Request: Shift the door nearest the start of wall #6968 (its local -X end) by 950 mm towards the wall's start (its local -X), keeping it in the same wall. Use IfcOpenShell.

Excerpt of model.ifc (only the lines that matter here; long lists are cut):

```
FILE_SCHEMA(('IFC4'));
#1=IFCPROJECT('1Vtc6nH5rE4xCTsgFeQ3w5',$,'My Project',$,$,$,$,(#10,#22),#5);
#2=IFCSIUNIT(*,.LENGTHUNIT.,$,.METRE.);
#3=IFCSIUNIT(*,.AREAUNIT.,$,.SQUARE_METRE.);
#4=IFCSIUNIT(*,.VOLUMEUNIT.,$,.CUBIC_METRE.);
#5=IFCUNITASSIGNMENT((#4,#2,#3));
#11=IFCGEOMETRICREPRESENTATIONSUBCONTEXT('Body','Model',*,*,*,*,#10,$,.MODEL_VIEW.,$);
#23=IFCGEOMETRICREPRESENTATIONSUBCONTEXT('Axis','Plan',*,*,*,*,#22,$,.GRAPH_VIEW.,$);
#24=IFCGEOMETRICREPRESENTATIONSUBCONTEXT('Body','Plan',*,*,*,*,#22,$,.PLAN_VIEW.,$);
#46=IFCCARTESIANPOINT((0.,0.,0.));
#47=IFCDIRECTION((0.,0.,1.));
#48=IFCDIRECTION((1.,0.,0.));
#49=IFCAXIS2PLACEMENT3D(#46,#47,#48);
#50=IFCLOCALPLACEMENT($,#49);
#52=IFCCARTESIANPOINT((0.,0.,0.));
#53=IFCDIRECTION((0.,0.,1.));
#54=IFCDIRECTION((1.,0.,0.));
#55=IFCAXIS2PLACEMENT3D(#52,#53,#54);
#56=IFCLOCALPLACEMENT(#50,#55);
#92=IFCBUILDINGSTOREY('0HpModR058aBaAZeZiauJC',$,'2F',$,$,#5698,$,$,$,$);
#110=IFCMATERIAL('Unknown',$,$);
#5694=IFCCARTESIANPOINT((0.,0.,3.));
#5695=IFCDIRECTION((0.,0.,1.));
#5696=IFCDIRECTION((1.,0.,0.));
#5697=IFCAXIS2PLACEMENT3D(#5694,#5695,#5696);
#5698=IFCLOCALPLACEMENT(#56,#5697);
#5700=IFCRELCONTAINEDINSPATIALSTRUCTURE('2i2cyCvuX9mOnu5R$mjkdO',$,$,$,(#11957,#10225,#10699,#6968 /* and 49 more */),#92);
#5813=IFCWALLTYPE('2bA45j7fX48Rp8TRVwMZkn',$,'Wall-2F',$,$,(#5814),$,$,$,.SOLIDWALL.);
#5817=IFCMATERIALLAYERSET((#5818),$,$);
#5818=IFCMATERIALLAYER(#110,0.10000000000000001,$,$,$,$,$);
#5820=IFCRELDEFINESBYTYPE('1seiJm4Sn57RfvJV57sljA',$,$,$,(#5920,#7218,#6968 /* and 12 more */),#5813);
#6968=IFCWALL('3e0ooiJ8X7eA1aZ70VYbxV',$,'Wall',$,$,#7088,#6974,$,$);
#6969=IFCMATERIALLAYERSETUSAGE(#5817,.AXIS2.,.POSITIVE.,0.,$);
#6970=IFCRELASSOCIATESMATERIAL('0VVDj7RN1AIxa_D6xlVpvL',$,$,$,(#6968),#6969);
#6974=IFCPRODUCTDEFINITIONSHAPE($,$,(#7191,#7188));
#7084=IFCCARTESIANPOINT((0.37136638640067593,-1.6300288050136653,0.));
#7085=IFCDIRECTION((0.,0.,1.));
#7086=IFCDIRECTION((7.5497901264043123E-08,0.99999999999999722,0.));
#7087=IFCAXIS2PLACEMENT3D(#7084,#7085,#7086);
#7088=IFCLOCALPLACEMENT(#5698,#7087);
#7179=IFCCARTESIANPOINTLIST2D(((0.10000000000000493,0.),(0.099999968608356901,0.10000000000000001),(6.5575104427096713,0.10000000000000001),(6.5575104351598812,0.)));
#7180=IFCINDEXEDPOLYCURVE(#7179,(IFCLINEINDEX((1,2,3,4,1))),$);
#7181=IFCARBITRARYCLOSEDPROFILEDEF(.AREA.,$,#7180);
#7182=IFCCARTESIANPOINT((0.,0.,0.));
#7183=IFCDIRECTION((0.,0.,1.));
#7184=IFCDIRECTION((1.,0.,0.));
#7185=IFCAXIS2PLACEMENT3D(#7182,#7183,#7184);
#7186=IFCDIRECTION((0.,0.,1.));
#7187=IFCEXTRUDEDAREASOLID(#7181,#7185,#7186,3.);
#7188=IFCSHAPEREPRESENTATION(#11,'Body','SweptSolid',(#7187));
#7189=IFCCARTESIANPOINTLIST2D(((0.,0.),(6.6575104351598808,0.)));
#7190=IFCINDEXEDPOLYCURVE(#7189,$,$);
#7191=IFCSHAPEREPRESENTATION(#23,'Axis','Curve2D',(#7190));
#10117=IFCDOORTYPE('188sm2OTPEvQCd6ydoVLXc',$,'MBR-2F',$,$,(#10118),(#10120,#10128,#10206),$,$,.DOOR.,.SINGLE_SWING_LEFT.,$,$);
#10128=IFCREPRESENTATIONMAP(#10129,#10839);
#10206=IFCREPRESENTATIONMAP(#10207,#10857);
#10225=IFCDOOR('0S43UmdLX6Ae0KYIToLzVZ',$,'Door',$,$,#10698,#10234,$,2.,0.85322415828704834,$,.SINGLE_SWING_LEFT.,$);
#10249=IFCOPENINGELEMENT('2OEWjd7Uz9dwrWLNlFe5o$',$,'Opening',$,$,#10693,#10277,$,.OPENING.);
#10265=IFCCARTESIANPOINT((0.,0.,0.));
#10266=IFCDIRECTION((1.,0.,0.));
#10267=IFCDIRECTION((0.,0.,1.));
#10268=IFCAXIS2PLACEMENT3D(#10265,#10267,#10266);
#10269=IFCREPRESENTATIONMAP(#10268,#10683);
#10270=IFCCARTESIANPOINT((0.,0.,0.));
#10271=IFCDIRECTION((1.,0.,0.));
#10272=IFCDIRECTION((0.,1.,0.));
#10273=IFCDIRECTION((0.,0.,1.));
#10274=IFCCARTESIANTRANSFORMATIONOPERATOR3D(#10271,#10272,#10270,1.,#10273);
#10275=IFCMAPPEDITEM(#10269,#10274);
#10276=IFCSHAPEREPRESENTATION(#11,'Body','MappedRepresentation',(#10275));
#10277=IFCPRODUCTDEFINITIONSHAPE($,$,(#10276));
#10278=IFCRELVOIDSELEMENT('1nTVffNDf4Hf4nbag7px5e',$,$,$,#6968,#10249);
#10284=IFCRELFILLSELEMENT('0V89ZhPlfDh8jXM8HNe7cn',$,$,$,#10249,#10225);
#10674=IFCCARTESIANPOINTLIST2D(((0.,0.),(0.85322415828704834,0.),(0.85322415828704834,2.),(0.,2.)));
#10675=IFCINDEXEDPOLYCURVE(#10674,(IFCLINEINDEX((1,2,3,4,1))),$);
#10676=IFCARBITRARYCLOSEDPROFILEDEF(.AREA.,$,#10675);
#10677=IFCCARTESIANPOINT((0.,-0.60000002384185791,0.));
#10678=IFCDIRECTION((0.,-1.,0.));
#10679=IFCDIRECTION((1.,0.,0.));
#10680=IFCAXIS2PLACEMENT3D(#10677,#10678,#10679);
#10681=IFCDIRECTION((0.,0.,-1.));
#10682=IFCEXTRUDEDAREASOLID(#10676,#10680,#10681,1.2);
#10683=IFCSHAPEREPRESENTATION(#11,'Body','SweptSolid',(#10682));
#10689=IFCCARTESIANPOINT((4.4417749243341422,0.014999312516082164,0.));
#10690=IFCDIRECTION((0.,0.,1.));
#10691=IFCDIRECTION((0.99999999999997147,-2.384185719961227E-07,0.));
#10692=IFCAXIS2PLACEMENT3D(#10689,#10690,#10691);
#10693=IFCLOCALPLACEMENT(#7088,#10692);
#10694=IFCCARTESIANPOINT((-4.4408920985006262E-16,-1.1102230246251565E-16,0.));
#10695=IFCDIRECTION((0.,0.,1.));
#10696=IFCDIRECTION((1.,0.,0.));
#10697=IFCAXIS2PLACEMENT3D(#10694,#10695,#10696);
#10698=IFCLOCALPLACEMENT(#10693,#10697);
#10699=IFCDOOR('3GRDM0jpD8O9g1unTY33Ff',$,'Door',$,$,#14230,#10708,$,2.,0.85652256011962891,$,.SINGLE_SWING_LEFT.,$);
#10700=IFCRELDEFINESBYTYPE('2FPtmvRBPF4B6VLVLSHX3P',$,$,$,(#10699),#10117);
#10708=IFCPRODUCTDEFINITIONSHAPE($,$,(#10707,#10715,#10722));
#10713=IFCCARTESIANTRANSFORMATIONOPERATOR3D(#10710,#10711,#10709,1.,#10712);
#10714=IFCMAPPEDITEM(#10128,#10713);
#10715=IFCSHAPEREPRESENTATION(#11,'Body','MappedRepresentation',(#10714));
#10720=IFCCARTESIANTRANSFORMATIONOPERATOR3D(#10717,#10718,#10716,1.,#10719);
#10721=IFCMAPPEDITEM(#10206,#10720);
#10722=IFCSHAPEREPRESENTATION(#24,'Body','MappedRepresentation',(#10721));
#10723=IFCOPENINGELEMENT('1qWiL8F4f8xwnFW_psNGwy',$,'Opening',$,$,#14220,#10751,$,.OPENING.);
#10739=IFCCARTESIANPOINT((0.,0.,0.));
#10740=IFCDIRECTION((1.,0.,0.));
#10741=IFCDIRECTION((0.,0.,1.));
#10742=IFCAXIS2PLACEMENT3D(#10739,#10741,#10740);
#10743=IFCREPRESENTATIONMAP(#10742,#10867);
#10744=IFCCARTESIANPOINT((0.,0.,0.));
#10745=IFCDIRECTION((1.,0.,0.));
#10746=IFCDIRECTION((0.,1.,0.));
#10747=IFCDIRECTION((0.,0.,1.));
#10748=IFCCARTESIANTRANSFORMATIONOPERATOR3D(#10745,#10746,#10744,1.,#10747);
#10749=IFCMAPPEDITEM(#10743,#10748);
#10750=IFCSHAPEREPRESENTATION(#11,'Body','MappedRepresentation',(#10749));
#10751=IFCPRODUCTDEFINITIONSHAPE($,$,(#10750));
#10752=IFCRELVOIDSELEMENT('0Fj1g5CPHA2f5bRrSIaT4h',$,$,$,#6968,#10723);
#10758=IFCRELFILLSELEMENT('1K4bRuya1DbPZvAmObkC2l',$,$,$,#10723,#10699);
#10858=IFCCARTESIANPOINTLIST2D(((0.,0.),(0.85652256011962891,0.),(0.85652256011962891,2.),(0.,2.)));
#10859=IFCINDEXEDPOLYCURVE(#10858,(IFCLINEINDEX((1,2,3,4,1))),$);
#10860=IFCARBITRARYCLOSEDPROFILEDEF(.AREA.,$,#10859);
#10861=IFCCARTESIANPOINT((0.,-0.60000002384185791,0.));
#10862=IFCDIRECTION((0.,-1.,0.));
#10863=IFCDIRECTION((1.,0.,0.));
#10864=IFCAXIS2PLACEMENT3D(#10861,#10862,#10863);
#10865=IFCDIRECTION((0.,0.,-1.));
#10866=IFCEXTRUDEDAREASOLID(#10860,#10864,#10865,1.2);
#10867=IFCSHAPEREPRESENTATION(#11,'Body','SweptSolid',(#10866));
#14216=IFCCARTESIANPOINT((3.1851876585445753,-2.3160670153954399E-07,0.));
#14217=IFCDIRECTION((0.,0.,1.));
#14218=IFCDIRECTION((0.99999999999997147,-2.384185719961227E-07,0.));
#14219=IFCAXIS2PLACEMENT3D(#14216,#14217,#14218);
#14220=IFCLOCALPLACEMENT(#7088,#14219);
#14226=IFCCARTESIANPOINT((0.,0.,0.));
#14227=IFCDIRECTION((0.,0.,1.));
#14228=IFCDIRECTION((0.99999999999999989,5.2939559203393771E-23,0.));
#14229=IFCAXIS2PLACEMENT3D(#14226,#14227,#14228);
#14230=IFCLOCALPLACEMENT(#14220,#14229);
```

```python
import ifcopenshell
import ifcopenshell.api.geometry
import ifcopenshell.util.placement

model = ifcopenshell.open("model.ifc")

door = model.by_id(10699)
opening = door.FillsVoids[0].RelatingOpeningElement
wall = opening.VoidsElements[0].RelatingBuildingElement

wall_matrix = ifcopenshell.util.placement.get_local_placement(wall.ObjectPlacement)
shift = wall_matrix[:3, 0] * -0.95
before = ifcopenshell.util.placement.get_local_placement(door.ObjectPlacement)[:3, 3].copy()

# The door is placed relative to its opening, so it follows when the opening moves.
matrix = ifcopenshell.util.placement.get_local_placement(opening.ObjectPlacement)
matrix[:3, 3] += shift
ifcopenshell.api.geometry.edit_object_placement(
    model, product=opening, matrix=matrix, is_si=False, should_transform_children=True
)

after = ifcopenshell.util.placement.get_local_placement(door.ObjectPlacement)[:3, 3]
print("door moved by", (after - before).round(3) + 0.0)

model.write("model_v2.ifc")
```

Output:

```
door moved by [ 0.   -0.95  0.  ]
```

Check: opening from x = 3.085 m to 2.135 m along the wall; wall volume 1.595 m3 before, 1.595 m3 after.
